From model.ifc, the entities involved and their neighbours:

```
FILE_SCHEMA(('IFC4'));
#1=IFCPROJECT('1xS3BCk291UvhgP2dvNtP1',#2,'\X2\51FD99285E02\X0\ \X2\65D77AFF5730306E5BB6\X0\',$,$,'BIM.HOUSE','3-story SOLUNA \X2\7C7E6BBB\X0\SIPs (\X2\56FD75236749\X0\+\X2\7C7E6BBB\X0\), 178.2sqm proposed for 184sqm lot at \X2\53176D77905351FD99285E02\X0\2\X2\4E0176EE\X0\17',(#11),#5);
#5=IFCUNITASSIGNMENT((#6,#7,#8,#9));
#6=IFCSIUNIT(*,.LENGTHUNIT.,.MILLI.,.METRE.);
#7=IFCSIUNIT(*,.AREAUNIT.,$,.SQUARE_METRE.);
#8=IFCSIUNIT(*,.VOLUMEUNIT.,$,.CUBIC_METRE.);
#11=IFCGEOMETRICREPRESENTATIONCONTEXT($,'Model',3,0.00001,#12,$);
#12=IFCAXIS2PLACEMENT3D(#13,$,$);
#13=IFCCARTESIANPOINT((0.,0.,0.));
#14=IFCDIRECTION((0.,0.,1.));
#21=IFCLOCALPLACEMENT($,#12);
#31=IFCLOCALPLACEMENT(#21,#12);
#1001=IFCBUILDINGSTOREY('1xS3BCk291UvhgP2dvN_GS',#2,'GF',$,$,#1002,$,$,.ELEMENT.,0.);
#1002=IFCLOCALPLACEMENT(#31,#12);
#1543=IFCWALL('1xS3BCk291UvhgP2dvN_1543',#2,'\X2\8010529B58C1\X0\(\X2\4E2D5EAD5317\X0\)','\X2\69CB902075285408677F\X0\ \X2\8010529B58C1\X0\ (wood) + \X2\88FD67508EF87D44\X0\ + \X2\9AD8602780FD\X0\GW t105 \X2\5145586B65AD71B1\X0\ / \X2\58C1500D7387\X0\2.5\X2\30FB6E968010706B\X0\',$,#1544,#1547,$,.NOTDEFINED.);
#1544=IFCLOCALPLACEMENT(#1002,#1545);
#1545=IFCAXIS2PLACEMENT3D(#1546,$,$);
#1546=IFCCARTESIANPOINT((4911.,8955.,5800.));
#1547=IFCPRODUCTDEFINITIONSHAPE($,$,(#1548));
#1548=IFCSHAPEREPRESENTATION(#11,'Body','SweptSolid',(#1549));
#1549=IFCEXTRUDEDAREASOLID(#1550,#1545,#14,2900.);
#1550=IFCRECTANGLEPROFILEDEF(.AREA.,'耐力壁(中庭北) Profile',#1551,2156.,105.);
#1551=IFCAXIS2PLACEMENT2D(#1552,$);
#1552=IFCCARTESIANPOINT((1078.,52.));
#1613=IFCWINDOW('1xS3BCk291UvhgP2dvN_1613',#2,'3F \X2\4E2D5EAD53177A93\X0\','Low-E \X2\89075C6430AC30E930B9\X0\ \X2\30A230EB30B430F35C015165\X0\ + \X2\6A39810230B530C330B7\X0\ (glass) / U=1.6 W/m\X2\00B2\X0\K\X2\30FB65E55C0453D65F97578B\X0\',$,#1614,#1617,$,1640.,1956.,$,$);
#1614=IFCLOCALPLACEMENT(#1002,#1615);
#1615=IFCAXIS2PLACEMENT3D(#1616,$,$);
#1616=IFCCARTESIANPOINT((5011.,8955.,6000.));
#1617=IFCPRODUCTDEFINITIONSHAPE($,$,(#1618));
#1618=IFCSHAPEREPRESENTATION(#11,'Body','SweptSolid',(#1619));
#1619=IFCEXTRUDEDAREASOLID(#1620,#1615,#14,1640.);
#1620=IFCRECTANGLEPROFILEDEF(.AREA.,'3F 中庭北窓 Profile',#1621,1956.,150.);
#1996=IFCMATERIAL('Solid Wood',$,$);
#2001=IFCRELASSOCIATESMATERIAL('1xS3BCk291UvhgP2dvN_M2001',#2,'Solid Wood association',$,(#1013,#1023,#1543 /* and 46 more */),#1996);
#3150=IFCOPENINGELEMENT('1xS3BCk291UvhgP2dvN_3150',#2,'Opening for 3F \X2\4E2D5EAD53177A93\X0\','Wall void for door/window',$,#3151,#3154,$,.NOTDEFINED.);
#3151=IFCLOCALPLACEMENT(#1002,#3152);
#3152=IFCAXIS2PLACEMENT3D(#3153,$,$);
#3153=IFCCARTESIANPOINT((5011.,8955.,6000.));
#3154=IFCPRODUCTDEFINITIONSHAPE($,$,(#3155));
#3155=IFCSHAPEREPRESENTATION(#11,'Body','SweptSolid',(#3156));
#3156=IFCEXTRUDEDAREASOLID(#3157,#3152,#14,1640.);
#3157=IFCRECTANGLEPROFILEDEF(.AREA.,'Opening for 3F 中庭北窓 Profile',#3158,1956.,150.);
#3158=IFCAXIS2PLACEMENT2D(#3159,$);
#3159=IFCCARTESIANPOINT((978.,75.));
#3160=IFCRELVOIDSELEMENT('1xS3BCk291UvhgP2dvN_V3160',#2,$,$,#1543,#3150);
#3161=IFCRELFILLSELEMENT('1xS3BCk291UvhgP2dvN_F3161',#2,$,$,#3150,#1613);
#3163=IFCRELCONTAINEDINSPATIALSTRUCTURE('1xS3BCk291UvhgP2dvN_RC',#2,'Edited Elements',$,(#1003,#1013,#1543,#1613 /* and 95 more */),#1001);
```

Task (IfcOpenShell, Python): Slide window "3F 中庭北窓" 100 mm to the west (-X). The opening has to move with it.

```python
import ifcopenshell
import ifcopenshell.api.geometry
import ifcopenshell.util.placement
import ifcopenshell.util.unit

model = ifcopenshell.open("model.ifc")
unit_scale = ifcopenshell.util.unit.calculate_unit_scale(model)

window = model.by_id(1613)
opening = window.FillsVoids[0].RelatingOpeningElement
wall = opening.VoidsElements[0].RelatingBuildingElement

wall_matrix = ifcopenshell.util.placement.get_local_placement(wall.ObjectPlacement)
shift = wall_matrix[:3, 0] * -0.1 / unit_scale
before = ifcopenshell.util.placement.get_local_placement(window.ObjectPlacement)[:3, 3].copy()

# The window is not placed relative to its opening, so move both.
for product in (opening, window):
    matrix = ifcopenshell.util.placement.get_local_placement(product.ObjectPlacement)
    matrix[:3, 3] += shift
    ifcopenshell.api.geometry.edit_object_placement(model, product=product, matrix=matrix, is_si=False)

after = ifcopenshell.util.placement.get_local_placement(window.ObjectPlacement)[:3, 3]
print("window moved by", (after - before).round(3) + 0.0)

model.write("model-out.ifc")
```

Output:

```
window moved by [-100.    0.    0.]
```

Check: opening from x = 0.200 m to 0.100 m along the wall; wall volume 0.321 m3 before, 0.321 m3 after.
